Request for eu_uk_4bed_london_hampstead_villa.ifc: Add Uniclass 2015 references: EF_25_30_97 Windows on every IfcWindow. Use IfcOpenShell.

First a look at what the model holds.

```python
import ifcopenshell

model = ifcopenshell.open("eu_uk_4bed_london_hampstead_villa.ifc")
print(model.schema)
print("classifications:", [c.Name for c in model.by_type("IfcClassification")])
for ifc_class in ("IfcDoor", "IfcRoof", "IfcStair", "IfcWall", "IfcWindow"):
    print(ifc_class, len(model.by_type(ifc_class)))
```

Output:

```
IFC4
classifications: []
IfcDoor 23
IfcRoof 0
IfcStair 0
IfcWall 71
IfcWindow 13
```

```python
import ifcopenshell
import ifcopenshell.api.classification

model = ifcopenshell.open("eu_uk_4bed_london_hampstead_villa.ifc")

system = ifcopenshell.api.classification.add_classification(model, classification="Uniclass 2015")

codes = {
    "IfcWindow": ("EF_25_30_97", "Windows"),
}
for ifc_class, (code, name) in codes.items():
    products = model.by_type(ifc_class)
    ifcopenshell.api.classification.add_reference(
        model, products=products, classification=system, identification=code, name=name
    )
    print(code, len(products))

model.write("eu_uk_4bed_london_hampstead_villa_updated.ifc")
```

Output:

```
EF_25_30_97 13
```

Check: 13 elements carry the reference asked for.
